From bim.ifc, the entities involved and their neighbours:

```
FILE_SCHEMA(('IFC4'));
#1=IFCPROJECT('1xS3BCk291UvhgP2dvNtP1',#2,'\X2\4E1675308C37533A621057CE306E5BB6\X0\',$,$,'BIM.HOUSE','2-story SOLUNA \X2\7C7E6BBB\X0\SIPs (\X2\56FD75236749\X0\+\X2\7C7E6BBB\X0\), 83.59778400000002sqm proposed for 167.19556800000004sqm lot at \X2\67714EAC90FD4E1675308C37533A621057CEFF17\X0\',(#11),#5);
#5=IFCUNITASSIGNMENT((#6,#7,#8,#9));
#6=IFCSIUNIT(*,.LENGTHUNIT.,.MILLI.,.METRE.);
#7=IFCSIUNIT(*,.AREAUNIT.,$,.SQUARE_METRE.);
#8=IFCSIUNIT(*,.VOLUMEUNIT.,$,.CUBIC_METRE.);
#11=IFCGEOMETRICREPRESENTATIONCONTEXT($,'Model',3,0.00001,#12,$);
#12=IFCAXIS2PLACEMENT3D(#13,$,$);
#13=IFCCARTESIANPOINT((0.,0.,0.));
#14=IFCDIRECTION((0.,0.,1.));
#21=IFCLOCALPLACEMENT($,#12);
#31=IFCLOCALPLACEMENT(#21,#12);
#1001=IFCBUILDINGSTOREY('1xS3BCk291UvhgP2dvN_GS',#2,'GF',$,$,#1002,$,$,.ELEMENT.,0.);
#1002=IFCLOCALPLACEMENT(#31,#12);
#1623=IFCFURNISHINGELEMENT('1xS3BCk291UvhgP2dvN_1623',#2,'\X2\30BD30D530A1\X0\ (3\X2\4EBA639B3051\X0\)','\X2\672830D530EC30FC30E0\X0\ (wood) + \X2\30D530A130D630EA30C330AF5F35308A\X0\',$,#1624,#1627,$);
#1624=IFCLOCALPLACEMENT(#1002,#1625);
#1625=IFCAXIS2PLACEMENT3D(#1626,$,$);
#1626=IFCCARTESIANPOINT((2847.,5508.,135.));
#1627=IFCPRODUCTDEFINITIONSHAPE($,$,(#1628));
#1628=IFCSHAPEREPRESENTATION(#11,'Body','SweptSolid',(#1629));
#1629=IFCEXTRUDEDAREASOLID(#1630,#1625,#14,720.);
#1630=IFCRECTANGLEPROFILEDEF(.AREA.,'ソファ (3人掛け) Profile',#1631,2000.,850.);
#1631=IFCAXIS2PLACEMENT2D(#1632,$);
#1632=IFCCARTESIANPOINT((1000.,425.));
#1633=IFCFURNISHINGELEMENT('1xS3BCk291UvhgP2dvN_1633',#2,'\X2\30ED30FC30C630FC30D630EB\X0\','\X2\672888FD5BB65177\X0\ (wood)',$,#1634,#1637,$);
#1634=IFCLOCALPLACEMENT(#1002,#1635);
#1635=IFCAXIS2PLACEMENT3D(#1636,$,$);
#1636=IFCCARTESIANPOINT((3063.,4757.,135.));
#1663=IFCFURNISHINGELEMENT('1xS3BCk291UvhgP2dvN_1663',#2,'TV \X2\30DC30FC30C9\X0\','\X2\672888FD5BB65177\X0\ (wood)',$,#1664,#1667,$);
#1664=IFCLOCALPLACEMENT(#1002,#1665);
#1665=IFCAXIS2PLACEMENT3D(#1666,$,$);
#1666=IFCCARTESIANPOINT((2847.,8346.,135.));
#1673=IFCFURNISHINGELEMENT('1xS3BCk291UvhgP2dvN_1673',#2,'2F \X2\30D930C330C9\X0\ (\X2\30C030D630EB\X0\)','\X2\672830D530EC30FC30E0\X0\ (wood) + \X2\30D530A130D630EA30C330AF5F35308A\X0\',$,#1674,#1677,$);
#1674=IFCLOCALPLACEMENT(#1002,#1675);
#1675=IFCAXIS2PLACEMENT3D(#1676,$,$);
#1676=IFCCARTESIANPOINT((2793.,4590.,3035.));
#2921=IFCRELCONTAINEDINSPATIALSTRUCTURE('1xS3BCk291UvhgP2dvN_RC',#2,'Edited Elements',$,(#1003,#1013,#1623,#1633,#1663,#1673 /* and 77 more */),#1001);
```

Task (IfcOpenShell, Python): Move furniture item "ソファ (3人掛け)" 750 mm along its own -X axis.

```python
import ifcopenshell
import ifcopenshell.api.geometry
import ifcopenshell.util.placement
import ifcopenshell.util.unit

model = ifcopenshell.open("bim.ifc")
unit_scale = ifcopenshell.util.unit.calculate_unit_scale(model)

item = model.by_guid("1xS3BCk291UvhgP2dvN_1623")
matrix = ifcopenshell.util.placement.get_local_placement(item.ObjectPlacement)
matrix[:3, 3] -= matrix[:3, 0] * 0.75 / unit_scale
ifcopenshell.api.geometry.edit_object_placement(model, product=item, matrix=matrix, is_si=False)

print(ifcopenshell.util.placement.get_local_placement(item.ObjectPlacement).round(3) + 0.0)

model.write("bim_edited.ifc")
```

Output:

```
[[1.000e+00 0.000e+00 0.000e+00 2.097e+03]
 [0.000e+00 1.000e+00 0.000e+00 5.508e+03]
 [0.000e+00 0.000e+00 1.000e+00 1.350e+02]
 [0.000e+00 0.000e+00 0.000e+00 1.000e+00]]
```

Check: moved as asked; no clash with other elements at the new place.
